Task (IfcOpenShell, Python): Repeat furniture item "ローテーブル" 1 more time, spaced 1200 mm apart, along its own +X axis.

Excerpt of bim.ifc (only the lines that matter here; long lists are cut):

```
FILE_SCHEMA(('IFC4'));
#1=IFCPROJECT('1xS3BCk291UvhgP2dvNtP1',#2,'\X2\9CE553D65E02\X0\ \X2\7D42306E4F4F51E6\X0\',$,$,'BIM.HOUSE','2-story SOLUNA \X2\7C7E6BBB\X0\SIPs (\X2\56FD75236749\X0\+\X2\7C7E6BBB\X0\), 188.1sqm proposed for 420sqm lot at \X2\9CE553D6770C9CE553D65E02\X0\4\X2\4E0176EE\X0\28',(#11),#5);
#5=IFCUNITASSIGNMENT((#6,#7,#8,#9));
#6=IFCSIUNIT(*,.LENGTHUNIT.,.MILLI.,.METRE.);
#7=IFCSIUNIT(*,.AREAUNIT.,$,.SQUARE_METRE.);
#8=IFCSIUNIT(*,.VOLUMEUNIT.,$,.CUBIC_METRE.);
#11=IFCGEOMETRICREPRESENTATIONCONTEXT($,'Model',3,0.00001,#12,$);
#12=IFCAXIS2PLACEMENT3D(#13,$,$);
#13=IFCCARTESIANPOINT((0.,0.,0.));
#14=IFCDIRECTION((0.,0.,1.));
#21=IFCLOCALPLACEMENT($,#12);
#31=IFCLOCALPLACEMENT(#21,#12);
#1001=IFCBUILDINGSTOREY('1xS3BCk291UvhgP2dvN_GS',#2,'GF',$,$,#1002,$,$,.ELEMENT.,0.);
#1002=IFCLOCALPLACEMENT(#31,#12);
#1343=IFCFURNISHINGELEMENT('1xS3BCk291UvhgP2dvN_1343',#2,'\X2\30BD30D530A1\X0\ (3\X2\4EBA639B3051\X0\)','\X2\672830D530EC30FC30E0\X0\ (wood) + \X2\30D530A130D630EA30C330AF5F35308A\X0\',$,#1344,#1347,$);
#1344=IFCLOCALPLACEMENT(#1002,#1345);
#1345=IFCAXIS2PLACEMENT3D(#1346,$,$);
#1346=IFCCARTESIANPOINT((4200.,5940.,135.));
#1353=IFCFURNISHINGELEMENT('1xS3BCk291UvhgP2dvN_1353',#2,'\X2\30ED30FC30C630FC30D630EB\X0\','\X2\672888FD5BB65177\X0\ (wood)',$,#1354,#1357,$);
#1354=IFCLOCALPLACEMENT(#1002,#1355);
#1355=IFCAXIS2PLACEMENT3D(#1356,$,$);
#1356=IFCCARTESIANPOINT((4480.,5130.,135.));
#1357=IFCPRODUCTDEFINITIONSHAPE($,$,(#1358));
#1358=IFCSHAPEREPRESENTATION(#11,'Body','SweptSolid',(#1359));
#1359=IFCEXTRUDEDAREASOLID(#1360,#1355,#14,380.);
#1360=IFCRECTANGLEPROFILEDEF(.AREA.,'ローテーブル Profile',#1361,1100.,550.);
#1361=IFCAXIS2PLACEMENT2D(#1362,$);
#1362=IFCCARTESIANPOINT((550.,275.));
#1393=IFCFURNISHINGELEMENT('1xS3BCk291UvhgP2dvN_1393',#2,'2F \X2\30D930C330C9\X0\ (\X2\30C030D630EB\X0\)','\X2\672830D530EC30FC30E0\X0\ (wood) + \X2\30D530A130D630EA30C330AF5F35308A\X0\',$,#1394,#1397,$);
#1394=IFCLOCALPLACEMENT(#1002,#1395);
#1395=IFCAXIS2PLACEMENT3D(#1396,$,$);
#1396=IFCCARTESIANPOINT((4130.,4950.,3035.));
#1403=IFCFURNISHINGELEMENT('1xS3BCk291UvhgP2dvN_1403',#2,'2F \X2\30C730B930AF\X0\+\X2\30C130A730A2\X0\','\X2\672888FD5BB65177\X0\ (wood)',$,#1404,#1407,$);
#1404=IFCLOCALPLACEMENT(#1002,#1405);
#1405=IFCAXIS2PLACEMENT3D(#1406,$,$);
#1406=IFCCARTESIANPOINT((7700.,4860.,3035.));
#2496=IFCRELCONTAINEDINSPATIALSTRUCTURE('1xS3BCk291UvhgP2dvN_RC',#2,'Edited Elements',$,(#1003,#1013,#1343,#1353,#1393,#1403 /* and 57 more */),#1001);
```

```python
import ifcopenshell
import ifcopenshell.api.geometry
import ifcopenshell.api.root
import ifcopenshell.util.element
import ifcopenshell.util.placement
import ifcopenshell.util.unit

model = ifcopenshell.open("bim.ifc")
unit_scale = ifcopenshell.util.unit.calculate_unit_scale(model)


def reuse_history(source, copy):
    """copy_class also copies each property set's owner history, people and application; keep the originals."""
    for rel in copy.IsDefinedBy:
        if rel.is_a("IfcRelDefinesByProperties") and (history := rel.RelatingPropertyDefinition.OwnerHistory):
            rel.RelatingPropertyDefinition.OwnerHistory = source.OwnerHistory
            ifcopenshell.util.element.remove_deep2(model, history)


source = model.by_id(1353)
base = ifcopenshell.util.placement.get_local_placement(source.ObjectPlacement)
step = base[:3, 0] * 1.2 / unit_scale

for i in range(1, 2):
    copy = ifcopenshell.api.root.copy_class(model, product=source)
    copy.Representation = ifcopenshell.util.element.copy_deep(
        model, source.Representation, exclude=["IfcGeometricRepresentationContext", "IfcRepresentationMap"]
    )
    reuse_history(source, copy)
    matrix = base.copy()
    matrix[:3, 3] += i * step
    print("added at", matrix[:3, 3].round(3) + 0.0)
    ifcopenshell.api.geometry.edit_object_placement(model, product=copy, matrix=matrix, is_si=False)

model.write("bim_rev.ifc")
```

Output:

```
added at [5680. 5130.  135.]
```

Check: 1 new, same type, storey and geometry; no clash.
